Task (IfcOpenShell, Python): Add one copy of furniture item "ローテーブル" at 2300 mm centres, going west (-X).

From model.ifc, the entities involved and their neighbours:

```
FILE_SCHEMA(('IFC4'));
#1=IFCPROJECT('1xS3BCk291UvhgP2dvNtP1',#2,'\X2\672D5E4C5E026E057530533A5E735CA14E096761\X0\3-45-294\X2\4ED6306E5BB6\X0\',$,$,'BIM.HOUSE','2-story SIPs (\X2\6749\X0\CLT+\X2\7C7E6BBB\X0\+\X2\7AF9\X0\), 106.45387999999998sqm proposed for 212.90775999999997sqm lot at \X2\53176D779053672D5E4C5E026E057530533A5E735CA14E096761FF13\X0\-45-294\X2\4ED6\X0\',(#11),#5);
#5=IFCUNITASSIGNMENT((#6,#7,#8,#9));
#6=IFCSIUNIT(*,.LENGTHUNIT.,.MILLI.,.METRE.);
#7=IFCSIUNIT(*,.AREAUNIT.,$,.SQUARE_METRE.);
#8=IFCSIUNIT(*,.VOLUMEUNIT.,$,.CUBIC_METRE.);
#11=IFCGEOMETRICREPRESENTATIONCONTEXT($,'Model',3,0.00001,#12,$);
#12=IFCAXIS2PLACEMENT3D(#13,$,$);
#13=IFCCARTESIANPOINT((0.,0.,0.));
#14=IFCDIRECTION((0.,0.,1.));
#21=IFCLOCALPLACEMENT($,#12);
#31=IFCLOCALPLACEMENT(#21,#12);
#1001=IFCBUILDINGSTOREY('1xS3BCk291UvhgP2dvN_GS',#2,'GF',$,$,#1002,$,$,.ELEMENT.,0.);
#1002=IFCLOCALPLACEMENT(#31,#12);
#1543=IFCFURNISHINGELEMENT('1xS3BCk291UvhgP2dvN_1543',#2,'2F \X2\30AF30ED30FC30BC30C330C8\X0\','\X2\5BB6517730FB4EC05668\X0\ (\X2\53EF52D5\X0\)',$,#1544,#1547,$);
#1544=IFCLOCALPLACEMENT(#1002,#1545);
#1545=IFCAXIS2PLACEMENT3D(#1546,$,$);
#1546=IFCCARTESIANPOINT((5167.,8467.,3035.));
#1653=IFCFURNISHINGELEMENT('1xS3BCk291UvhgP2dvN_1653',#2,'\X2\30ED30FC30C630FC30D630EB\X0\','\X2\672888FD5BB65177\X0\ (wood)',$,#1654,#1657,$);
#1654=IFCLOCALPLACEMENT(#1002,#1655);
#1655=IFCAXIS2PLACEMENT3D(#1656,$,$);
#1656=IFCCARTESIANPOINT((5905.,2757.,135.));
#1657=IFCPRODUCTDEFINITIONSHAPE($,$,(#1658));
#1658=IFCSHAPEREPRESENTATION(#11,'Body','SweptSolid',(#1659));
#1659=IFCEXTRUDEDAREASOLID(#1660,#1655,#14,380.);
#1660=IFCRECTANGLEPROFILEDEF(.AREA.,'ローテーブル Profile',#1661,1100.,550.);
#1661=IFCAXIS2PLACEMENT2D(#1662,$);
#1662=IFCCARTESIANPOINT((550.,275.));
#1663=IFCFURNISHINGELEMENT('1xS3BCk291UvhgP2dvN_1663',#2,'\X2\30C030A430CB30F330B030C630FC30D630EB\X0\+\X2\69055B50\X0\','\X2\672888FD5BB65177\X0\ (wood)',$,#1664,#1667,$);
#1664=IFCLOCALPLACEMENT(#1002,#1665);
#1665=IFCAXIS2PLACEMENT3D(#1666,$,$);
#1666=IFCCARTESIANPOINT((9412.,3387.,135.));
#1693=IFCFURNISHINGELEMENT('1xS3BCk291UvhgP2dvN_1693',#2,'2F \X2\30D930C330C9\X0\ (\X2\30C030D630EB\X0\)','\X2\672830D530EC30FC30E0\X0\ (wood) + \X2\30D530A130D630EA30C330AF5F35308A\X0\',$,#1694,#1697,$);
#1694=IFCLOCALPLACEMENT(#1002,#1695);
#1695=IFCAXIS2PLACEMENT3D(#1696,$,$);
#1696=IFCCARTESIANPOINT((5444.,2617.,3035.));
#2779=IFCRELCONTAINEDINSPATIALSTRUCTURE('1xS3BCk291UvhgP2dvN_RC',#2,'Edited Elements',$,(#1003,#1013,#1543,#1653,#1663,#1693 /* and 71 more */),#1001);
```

```python
import numpy as np
import ifcopenshell
import ifcopenshell.api.geometry
import ifcopenshell.api.root
import ifcopenshell.util.element
import ifcopenshell.util.placement
import ifcopenshell.util.unit

model = ifcopenshell.open("model.ifc")
unit_scale = ifcopenshell.util.unit.calculate_unit_scale(model)


def reuse_history(source, copy):
    """copy_class also copies each property set's owner history, people and application; keep the originals."""
    for rel in copy.IsDefinedBy:
        if rel.is_a("IfcRelDefinesByProperties") and (history := rel.RelatingPropertyDefinition.OwnerHistory):
            rel.RelatingPropertyDefinition.OwnerHistory = source.OwnerHistory
            ifcopenshell.util.element.remove_deep2(model, history)


source = model.by_guid("1xS3BCk291UvhgP2dvN_1653")
base = ifcopenshell.util.placement.get_local_placement(source.ObjectPlacement)
step = np.array([-1.0, 0.0, 0.0]) * 2.3 / unit_scale

for i in range(1, 2):
    copy = ifcopenshell.api.root.copy_class(model, product=source)
    copy.Representation = ifcopenshell.util.element.copy_deep(
        model, source.Representation, exclude=["IfcGeometricRepresentationContext", "IfcRepresentationMap"]
    )
    reuse_history(source, copy)
    matrix = base.copy()
    matrix[:3, 3] += i * step
    print("added at", matrix[:3, 3].round(3) + 0.0)
    ifcopenshell.api.geometry.edit_object_placement(model, product=copy, matrix=matrix, is_si=False)

model.write("model_updated.ifc")
```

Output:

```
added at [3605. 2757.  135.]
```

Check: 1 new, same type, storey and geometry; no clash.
